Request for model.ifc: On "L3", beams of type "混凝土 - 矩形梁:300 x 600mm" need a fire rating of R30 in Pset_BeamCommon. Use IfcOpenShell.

First a look at what the model holds.

```python
import ifcopenshell
import ifcopenshell.util.element

model = ifcopenshell.open("model.ifc")
print(model.schema)
storey = next(s for s in model.by_type("IfcBuildingStorey") if s.Name == "L3")
beams = [e for e in ifcopenshell.util.element.get_decomposition(storey) if e.is_a("IfcBeam")]
seen = {}
for e in beams:
    element_type = ifcopenshell.util.element.get_type(e)
    key = (element_type.Name if element_type != e and element_type else None, ifcopenshell.util.element.get_pset(e, "Pset_BeamCommon", "FireRating"))
    seen[key] = seen.get(key, 0) + 1
for (name, value), count in sorted(seen.items(), key=str):
    print(count, "x", name, "|", value)
```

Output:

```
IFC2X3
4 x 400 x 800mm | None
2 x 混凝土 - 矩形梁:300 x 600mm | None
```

```python
import ifcopenshell
import ifcopenshell.api.pset
import ifcopenshell.util.element

model = ifcopenshell.open("model.ifc")

storey = next(s for s in model.by_type("IfcBuildingStorey") if s.Name == "L3")
beams = [e for e in ifcopenshell.util.element.get_decomposition(storey) if e.is_a("IfcBeam")]

count = 0
for e in beams:
    element_type = ifcopenshell.util.element.get_type(e)
    if element_type in (None, e) or element_type.Name != "混凝土 - 矩形梁:300 x 600mm":
        continue
    # add_pset returns the element's existing set when there is one.
    pset = ifcopenshell.api.pset.add_pset(model, product=e, name="Pset_BeamCommon")
    ifcopenshell.api.pset.edit_pset(model, pset=pset, properties={"FireRating": "R30"})
    count += 1

print(count, "beams updated")

model.write("model_edited.ifc")
```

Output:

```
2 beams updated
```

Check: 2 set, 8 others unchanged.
